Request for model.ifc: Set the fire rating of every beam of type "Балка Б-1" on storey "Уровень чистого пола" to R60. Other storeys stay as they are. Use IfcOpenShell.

First a look at what the model holds.

```python
import ifcopenshell
import ifcopenshell.util.element

model = ifcopenshell.open("model.ifc")
print(model.schema)
storey = next(s for s in model.by_type("IfcBuildingStorey") if s.Name == "Уровень чистого пола")
beams = [e for e in ifcopenshell.util.element.get_decomposition(storey) if e.is_a("IfcBeam")]
seen = {}
for e in beams:
    element_type = ifcopenshell.util.element.get_type(e)
    key = (element_type.Name if element_type != e and element_type else None, ifcopenshell.util.element.get_pset(e, "Pset_BeamCommon", "FireRating"))
    seen[key] = seen.get(key, 0) + 1
for (name, value), count in sorted(seen.items(), key=str):
    print(count, "x", name, "|", value)
```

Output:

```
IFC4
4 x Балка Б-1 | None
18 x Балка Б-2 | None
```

```python
import ifcopenshell
import ifcopenshell.api.pset
import ifcopenshell.util.element

model = ifcopenshell.open("model.ifc")

storey = next(s for s in model.by_type("IfcBuildingStorey") if s.Name == "Уровень чистого пола")
beams = [e for e in ifcopenshell.util.element.get_decomposition(storey) if e.is_a("IfcBeam")]

count = 0
for e in beams:
    element_type = ifcopenshell.util.element.get_type(e)
    if element_type in (None, e) or element_type.Name != "Балка Б-1":
        continue
    # add_pset returns the element's existing set when there is one.
    pset = ifcopenshell.api.pset.add_pset(model, product=e, name="Pset_BeamCommon")
    ifcopenshell.api.pset.edit_pset(model, pset=pset, properties={"FireRating": "R60"})
    count += 1

print(count, "beams updated")

model.write("model_updated.ifc")
```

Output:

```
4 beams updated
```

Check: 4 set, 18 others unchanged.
